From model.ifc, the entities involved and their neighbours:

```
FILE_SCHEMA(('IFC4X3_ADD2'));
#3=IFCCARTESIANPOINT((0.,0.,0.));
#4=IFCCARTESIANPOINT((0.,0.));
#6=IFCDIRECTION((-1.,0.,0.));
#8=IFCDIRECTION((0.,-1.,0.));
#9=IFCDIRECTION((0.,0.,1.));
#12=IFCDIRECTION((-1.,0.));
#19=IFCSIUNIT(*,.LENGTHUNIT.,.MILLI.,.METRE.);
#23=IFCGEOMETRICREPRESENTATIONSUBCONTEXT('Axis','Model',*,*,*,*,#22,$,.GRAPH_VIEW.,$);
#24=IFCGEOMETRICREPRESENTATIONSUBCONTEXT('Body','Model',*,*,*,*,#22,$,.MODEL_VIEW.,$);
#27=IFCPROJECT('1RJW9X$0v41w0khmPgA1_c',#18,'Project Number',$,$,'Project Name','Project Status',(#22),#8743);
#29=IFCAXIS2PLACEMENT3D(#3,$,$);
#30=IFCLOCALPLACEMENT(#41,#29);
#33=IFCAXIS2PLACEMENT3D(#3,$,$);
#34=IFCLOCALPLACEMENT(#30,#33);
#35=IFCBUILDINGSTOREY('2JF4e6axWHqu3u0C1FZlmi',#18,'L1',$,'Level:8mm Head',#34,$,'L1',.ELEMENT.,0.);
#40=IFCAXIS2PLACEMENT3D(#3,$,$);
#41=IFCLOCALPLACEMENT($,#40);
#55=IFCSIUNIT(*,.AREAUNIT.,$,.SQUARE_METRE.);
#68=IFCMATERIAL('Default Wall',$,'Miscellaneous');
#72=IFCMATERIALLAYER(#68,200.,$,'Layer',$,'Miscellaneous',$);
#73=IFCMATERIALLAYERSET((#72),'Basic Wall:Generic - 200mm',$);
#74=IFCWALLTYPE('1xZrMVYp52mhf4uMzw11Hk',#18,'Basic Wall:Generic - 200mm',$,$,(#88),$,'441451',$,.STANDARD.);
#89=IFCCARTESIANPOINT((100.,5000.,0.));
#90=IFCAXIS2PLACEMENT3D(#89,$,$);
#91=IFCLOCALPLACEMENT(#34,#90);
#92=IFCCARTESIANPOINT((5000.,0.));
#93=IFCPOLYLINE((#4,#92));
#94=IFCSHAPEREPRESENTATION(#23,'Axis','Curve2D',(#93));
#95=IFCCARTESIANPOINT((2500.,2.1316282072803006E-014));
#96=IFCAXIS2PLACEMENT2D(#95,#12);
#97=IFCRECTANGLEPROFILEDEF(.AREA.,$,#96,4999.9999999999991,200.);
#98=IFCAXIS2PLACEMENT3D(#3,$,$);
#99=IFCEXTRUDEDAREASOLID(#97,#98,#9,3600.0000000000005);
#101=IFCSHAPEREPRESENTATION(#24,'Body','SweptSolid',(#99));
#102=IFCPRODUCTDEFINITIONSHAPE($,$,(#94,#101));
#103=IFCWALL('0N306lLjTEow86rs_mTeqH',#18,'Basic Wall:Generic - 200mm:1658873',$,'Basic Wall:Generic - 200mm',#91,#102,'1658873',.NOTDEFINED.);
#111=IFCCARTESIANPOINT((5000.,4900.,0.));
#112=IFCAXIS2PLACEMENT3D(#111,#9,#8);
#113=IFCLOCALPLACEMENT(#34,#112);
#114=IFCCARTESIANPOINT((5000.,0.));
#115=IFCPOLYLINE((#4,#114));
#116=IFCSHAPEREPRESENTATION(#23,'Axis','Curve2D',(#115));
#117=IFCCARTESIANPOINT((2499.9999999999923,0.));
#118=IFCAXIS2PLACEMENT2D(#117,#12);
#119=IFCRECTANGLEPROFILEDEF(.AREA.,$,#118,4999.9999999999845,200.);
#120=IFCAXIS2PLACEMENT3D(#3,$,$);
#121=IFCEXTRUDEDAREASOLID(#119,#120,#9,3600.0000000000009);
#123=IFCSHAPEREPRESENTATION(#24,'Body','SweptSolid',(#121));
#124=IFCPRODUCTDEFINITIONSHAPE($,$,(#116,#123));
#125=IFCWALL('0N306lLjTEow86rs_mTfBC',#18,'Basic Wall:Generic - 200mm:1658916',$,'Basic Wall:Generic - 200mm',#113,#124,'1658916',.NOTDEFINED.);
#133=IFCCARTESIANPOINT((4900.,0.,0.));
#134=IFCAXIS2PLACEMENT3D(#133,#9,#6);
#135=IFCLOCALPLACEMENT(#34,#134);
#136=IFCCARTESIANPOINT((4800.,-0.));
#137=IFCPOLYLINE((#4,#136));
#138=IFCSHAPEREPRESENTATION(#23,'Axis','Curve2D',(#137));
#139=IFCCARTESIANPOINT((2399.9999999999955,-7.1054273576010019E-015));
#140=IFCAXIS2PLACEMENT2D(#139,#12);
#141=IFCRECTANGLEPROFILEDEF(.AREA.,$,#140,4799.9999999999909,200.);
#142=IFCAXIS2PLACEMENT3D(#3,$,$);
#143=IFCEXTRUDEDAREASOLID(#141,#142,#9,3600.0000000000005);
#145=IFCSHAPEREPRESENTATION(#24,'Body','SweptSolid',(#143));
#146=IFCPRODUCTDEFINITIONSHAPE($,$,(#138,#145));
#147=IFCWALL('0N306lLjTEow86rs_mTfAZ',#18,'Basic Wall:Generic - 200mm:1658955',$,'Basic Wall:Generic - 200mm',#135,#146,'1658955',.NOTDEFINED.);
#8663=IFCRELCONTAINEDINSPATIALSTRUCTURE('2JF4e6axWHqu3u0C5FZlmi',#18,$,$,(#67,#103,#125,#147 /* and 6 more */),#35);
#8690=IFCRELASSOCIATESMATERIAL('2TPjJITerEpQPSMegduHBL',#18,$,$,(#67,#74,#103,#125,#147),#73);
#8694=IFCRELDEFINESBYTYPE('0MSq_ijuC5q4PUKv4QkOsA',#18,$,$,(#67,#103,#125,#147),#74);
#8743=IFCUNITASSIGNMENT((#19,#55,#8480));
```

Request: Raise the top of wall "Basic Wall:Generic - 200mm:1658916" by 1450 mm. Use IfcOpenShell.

```python
import ifcopenshell
import ifcopenshell.geom
import ifcopenshell.util.representation
import ifcopenshell.util.shape

model = ifcopenshell.open("model.ifc")
settings = ifcopenshell.geom.settings()


def volume(element):
    """Net volume in cubic metres, openings subtracted."""
    shape = ifcopenshell.geom.create_shape(settings, element)
    return ifcopenshell.util.shape.get_volume(shape.geometry)


wall = model.by_id(125)
before = volume(wall)

body = ifcopenshell.util.representation.get_representation(wall, "Model", "Body")
solid = body.Items[0]
old_height = solid.Depth
solid.Depth += 1450.0
after = volume(wall)

print(f"height {old_height:g} -> {solid.Depth:g}, volume {before:.3f} -> {after:.3f} m3")

model.write("model_edited.ifc")
```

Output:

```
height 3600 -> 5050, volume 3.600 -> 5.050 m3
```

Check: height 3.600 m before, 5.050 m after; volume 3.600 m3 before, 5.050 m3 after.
